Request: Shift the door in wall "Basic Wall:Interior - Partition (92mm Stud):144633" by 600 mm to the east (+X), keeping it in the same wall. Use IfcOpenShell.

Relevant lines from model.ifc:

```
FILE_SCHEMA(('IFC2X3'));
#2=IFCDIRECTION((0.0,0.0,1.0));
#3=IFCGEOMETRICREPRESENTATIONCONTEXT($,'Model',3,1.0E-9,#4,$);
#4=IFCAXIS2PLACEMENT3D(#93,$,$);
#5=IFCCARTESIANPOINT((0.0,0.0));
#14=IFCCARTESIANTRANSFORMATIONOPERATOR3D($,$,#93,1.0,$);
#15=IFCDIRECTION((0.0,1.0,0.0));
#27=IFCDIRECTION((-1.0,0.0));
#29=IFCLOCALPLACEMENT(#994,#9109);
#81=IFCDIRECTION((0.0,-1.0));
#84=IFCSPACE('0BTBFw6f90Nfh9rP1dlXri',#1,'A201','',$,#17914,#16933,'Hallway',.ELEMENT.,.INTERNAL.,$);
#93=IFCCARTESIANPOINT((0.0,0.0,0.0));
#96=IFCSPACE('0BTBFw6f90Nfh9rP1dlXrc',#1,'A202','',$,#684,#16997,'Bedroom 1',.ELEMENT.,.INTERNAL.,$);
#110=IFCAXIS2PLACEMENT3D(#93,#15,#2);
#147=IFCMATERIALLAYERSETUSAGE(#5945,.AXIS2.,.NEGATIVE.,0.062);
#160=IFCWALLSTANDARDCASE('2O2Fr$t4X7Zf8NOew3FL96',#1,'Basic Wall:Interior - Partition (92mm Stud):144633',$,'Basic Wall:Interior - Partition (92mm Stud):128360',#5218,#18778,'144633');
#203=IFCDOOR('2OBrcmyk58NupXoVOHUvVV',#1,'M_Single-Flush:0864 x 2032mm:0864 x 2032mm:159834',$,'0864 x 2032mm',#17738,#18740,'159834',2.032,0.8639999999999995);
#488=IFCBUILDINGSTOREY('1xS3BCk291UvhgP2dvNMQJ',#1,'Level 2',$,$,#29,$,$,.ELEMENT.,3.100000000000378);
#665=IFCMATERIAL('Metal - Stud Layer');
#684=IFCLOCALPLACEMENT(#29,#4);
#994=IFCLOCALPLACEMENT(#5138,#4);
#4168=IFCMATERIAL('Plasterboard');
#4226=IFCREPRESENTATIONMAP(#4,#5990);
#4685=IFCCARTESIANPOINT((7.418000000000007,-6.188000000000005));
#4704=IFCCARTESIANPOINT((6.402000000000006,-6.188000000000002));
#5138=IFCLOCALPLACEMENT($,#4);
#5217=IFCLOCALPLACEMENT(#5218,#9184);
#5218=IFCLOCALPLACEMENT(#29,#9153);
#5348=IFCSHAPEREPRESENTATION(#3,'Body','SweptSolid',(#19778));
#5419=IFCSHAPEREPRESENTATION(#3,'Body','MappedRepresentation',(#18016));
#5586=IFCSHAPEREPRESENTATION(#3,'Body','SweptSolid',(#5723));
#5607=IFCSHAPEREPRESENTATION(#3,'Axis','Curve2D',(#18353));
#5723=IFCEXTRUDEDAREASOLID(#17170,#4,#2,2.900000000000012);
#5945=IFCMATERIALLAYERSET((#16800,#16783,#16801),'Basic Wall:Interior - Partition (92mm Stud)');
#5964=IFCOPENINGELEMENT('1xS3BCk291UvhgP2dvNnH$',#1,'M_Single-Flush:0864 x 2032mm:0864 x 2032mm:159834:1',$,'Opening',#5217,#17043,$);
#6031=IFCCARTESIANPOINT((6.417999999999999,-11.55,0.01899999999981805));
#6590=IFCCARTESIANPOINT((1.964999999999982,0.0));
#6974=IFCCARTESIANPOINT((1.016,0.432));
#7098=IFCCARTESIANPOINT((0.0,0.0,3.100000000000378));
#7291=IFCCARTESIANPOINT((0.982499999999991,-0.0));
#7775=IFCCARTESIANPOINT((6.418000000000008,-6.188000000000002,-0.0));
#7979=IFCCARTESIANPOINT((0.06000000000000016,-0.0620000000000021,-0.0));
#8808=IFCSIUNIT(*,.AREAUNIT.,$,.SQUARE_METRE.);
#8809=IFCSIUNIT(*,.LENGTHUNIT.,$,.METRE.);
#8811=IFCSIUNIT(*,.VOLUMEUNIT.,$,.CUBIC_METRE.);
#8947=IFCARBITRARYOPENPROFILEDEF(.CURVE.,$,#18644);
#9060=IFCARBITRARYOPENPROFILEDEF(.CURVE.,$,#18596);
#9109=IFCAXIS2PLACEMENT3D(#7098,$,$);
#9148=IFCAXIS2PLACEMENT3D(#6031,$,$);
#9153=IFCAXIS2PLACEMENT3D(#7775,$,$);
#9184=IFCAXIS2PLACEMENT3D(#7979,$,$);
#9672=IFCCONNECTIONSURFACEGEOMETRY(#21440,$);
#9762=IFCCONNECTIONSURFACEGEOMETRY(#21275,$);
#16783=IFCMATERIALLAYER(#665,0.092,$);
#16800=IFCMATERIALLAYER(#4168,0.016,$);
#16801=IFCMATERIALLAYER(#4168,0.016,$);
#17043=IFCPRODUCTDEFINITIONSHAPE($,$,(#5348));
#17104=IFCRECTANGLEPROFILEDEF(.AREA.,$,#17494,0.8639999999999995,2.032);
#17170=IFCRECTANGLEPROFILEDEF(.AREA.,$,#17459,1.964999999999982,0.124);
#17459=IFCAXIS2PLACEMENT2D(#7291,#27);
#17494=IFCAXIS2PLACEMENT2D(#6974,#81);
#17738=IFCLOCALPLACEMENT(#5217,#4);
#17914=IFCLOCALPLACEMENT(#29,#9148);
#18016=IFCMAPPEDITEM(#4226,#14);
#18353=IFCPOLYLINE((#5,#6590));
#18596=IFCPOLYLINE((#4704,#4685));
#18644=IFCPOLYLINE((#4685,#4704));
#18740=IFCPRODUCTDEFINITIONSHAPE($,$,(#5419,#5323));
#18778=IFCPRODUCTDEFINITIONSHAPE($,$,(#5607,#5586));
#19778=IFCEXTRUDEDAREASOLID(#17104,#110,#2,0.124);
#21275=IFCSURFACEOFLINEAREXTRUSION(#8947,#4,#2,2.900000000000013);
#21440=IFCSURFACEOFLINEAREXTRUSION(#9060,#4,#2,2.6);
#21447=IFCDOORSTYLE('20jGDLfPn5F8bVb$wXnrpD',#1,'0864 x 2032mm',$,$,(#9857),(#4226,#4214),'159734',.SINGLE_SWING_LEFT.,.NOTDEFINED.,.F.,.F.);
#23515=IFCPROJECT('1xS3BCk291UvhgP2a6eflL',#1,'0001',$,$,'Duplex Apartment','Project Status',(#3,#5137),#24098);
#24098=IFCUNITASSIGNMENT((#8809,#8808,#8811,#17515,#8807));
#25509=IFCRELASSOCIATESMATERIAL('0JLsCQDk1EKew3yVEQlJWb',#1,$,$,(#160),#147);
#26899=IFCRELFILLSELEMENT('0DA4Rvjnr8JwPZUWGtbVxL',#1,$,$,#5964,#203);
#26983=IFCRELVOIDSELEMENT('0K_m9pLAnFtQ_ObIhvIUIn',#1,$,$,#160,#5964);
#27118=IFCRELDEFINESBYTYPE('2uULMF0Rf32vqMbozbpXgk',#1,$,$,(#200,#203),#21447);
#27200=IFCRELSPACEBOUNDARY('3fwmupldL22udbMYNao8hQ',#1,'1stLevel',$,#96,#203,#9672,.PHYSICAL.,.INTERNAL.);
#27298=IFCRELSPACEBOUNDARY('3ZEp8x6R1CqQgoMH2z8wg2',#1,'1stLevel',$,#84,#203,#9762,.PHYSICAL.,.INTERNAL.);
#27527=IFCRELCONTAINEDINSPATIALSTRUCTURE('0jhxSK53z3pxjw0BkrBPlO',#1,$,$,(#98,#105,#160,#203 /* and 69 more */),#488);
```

```python
import numpy as np
import ifcopenshell
import ifcopenshell.api.geometry
import ifcopenshell.util.placement

model = ifcopenshell.open("model.ifc")

door = model.by_guid("2OBrcmyk58NupXoVOHUvVV")
opening = door.FillsVoids[0].RelatingOpeningElement
wall = opening.VoidsElements[0].RelatingBuildingElement

wall_matrix = ifcopenshell.util.placement.get_local_placement(wall.ObjectPlacement)
shift = wall_matrix[:3, 0] * 0.6
before = ifcopenshell.util.placement.get_local_placement(door.ObjectPlacement)[:3, 3].copy()

# The door is placed relative to its opening, so it follows when the opening moves.
matrix = ifcopenshell.util.placement.get_local_placement(opening.ObjectPlacement)
matrix[:3, 3] += shift
ifcopenshell.api.geometry.edit_object_placement(
    model, product=opening, matrix=matrix, is_si=False, should_transform_children=True
)

# Space boundary surfaces are stored in each space's coordinates; move them too.
for rel in door.ProvidesBoundaries:
    if not rel.ConnectionGeometry:
        continue
    surface = rel.ConnectionGeometry.SurfaceOnRelatingElement
    space_matrix = ifcopenshell.util.placement.get_local_placement(rel.RelatingSpace.ObjectPlacement)
    point = np.array(surface.Position.Location.Coordinates) + space_matrix[:3, :3].T @ shift
    surface.Position = model.createIfcAxis2Placement3D(
        model.createIfcCartesianPoint(point.tolist()), surface.Position.Axis, surface.Position.RefDirection
    )

after = ifcopenshell.util.placement.get_local_placement(door.ObjectPlacement)[:3, 3]
print("door moved by", (after - before).round(3) + 0.0)

model.write("model-out.ifc")
```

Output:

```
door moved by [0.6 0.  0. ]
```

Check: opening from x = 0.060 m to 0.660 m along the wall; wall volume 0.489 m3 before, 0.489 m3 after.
